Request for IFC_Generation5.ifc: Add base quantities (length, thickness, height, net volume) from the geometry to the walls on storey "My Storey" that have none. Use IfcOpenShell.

First a look at what the model holds.

```python
import ifcopenshell
import ifcopenshell.util.element
import ifcopenshell.util.unit

model = ifcopenshell.open("IFC_Generation5.ifc")
print(model.schema)
for unit_type in ("LENGTHUNIT", "AREAUNIT", "VOLUMEUNIT"):
    print(unit_type, ifcopenshell.util.unit.calculate_unit_scale(model, unit_type))
storey = next(s for s in model.by_type("IfcBuildingStorey") if s.Name == "My Storey")
walls = [e for e in ifcopenshell.util.element.get_decomposition(storey) if e.is_a("IfcWall")]
for e in sorted(walls, key=lambda e: e.id()):
    print(e.id(), e.is_a(), e.Name, list(ifcopenshell.util.element.get_psets(e, qtos_only=True)), sep=" | ")
```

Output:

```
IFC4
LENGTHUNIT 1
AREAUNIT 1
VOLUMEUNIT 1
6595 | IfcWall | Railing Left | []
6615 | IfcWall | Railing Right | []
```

```python
import ifcopenshell
import ifcopenshell.api.pset
import ifcopenshell.geom
import ifcopenshell.util.element
import ifcopenshell.util.shape
import ifcopenshell.util.unit

model = ifcopenshell.open("IFC_Generation5.ifc")
unit_scale = ifcopenshell.util.unit.calculate_unit_scale(model)
volume_scale = ifcopenshell.util.unit.calculate_unit_scale(model, "VOLUMEUNIT")
settings = ifcopenshell.geom.settings()

storey = next(s for s in model.by_type("IfcBuildingStorey") if s.Name == "My Storey")
walls = [e for e in ifcopenshell.util.element.get_decomposition(storey) if e.is_a("IfcWall")]

for e in sorted(walls, key=lambda e: e.id()):
    if ifcopenshell.util.element.get_psets(e, qtos_only=True, should_inherit=False):
        continue
    # Geometry comes back in metres, in the element's own axes.
    shape = ifcopenshell.geom.create_shape(settings, e)
    values = {
        "Length": ifcopenshell.util.shape.get_x(shape.geometry) / unit_scale,
        "Width": ifcopenshell.util.shape.get_y(shape.geometry) / unit_scale,
        "Height": ifcopenshell.util.shape.get_z(shape.geometry) / unit_scale,
        "NetVolume": ifcopenshell.util.shape.get_volume(shape.geometry) / volume_scale,
    }
    qto = ifcopenshell.api.pset.add_qto(model, product=e, name="Qto_WallBaseQuantities")
    ifcopenshell.api.pset.edit_qto(model, qto=qto, properties=values)
    print(e.id(), {k: round(v, 3) for k, v in values.items()})

model.write("IFC_Generation5-out.ifc")
```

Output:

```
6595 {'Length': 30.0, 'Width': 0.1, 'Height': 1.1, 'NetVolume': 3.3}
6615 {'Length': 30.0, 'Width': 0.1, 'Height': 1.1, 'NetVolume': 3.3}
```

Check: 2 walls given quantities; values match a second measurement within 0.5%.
